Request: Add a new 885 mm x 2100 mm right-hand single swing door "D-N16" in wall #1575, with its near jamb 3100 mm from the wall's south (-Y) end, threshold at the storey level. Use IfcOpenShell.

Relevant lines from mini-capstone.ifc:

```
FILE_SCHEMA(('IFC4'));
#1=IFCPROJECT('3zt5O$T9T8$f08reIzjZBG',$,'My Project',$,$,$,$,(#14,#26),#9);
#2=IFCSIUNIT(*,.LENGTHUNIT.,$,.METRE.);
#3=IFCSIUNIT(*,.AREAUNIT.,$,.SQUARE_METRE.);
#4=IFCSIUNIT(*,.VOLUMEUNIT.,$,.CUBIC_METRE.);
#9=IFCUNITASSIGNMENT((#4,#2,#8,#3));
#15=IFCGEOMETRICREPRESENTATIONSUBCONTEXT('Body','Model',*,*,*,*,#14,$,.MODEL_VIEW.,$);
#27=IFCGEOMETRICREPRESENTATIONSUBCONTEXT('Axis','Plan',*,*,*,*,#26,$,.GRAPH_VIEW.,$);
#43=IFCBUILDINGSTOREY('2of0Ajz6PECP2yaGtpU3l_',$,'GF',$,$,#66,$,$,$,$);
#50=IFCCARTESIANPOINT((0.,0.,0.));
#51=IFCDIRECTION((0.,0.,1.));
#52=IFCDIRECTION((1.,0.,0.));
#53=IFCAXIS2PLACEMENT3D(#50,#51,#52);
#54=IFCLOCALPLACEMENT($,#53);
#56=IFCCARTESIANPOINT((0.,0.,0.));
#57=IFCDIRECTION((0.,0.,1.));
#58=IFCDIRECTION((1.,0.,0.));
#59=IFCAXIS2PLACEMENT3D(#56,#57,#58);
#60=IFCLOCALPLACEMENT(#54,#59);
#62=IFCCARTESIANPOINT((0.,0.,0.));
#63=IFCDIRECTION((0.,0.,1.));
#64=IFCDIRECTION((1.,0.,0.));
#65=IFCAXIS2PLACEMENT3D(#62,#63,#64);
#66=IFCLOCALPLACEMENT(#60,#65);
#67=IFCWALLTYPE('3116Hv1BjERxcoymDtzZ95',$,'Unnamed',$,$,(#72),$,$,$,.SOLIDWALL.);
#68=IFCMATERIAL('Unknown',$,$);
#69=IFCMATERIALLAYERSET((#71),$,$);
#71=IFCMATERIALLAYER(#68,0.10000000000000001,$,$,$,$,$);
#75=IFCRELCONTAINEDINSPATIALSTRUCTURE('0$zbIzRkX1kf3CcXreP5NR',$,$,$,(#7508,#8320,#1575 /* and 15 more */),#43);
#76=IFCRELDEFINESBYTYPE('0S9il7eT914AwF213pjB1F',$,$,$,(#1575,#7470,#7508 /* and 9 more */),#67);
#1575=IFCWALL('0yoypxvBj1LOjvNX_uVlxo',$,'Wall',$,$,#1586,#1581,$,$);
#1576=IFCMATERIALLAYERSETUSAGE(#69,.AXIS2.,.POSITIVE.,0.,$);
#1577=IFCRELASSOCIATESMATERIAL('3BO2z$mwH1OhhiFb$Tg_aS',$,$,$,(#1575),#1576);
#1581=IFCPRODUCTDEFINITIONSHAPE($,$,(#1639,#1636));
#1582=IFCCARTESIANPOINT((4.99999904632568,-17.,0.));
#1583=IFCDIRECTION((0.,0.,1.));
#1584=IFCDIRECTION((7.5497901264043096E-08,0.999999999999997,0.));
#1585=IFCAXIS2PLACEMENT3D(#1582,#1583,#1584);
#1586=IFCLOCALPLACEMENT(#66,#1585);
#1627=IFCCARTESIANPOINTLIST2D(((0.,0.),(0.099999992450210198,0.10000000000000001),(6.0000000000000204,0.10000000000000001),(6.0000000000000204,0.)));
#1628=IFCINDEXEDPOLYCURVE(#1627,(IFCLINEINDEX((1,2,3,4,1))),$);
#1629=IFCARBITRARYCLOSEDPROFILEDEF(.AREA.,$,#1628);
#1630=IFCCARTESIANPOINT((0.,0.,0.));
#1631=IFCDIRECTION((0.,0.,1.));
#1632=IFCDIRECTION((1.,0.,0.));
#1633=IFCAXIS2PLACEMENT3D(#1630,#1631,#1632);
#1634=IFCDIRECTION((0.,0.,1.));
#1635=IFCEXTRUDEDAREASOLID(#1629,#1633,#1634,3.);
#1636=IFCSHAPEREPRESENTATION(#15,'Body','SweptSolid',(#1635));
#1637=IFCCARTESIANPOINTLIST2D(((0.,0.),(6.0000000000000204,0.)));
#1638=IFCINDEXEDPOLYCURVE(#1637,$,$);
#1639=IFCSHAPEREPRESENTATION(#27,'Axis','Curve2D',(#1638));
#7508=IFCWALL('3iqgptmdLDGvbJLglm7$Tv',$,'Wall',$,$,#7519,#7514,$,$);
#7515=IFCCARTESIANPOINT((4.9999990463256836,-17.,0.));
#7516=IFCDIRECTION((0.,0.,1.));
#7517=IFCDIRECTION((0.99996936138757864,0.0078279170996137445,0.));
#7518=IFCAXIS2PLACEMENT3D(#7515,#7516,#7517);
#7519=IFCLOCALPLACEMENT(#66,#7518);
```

```python
import numpy as np
import ifcopenshell
import ifcopenshell.api.feature
import ifcopenshell.api.geometry
import ifcopenshell.api.root
import ifcopenshell.api.spatial
import ifcopenshell.geom
import ifcopenshell.util.element
import ifcopenshell.util.placement
import ifcopenshell.util.representation
import ifcopenshell.util.shape
import ifcopenshell.util.unit

model = ifcopenshell.open("mini-capstone.ifc")
unit_scale = ifcopenshell.util.unit.calculate_unit_scale(model)
settings = ifcopenshell.geom.settings()


def volume(element):
    """Net volume in cubic metres, openings subtracted."""
    shape = ifcopenshell.geom.create_shape(settings, element)
    return ifcopenshell.util.shape.get_volume(shape.geometry)


wall = model.by_id(1575)
storey = ifcopenshell.util.element.get_container(wall, ifc_class="IfcBuildingStorey")
context = ifcopenshell.util.representation.get_context(model, "Model", "Body", "MODEL_VIEW")
before = volume(wall)

width, height, from_end, sill = 0.885, 2.1, 3.1, 0.0  # metres

# The wall runs along its own X axis, and the end named is its -X end.
wall_shape = ifcopenshell.geom.create_shape(settings, wall)
x, y, z = ifcopenshell.util.shape.get_vertices(wall_shape.geometry).T
start = x.min() + from_end
face, thickness = float(y.min()), float(y.max() - y.min())
wall_matrix = ifcopenshell.util.placement.get_local_placement(wall.ObjectPlacement)
level = ifcopenshell.util.placement.get_local_placement(storey.ObjectPlacement)[2, 3]


def in_wall(x, y):
    """Placement at x, y metres in the wall's axes, at sill height."""
    matrix = wall_matrix.copy()
    matrix[:, 3] = wall_matrix @ np.array([x / unit_scale, y / unit_scale, 0.0, 1.0])
    matrix[2, 3] = level + sill / unit_scale
    return matrix


# Opening: a box that overshoots both wall faces by 50 mm.
opening = ifcopenshell.api.root.create_entity(model, ifc_class="IfcOpeningElement", predefined_type="OPENING")
box = ifcopenshell.api.geometry.add_wall_representation(
    model, context=context, length=width, height=height, thickness=thickness + 0.1
)
ifcopenshell.api.geometry.assign_representation(model, product=opening, representation=box)
ifcopenshell.api.geometry.edit_object_placement(model, product=opening, matrix=in_wall(start, face - 0.05), is_si=False)
ifcopenshell.api.feature.add_feature(model, feature=opening, element=wall)

door = ifcopenshell.api.root.create_entity(model, ifc_class="IfcDoor", name="D-N16", predefined_type="DOOR")
door.OverallWidth, door.OverallHeight = width / unit_scale, height / unit_scale
door.OperationType = "SINGLE_SWING_RIGHT"
body = ifcopenshell.api.geometry.add_door_representation(
    model,
    context=context,
    overall_width=door.OverallWidth,
    overall_height=door.OverallHeight,
    operation_type="SINGLE_SWING_RIGHT",
    lining_properties={"LiningDepth": thickness / unit_scale, "ThresholdDepth": thickness / unit_scale},
)
ifcopenshell.api.geometry.assign_representation(model, product=door, representation=body)
ifcopenshell.api.spatial.assign_container(model, products=[door], relating_structure=storey)
ifcopenshell.api.feature.add_filling(model, opening=opening, element=door)

# The lining spans the wall, so the door starts at the wall face.
ifcopenshell.api.geometry.edit_object_placement(model, product=door, matrix=in_wall(start, face), is_si=False)

after = volume(wall)

print(f"wall volume {before:.3f} -> {after:.3f} m3")

model.write("mini-capstone_edited.ifc")
```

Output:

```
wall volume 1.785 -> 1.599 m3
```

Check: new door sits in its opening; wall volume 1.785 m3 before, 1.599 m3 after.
